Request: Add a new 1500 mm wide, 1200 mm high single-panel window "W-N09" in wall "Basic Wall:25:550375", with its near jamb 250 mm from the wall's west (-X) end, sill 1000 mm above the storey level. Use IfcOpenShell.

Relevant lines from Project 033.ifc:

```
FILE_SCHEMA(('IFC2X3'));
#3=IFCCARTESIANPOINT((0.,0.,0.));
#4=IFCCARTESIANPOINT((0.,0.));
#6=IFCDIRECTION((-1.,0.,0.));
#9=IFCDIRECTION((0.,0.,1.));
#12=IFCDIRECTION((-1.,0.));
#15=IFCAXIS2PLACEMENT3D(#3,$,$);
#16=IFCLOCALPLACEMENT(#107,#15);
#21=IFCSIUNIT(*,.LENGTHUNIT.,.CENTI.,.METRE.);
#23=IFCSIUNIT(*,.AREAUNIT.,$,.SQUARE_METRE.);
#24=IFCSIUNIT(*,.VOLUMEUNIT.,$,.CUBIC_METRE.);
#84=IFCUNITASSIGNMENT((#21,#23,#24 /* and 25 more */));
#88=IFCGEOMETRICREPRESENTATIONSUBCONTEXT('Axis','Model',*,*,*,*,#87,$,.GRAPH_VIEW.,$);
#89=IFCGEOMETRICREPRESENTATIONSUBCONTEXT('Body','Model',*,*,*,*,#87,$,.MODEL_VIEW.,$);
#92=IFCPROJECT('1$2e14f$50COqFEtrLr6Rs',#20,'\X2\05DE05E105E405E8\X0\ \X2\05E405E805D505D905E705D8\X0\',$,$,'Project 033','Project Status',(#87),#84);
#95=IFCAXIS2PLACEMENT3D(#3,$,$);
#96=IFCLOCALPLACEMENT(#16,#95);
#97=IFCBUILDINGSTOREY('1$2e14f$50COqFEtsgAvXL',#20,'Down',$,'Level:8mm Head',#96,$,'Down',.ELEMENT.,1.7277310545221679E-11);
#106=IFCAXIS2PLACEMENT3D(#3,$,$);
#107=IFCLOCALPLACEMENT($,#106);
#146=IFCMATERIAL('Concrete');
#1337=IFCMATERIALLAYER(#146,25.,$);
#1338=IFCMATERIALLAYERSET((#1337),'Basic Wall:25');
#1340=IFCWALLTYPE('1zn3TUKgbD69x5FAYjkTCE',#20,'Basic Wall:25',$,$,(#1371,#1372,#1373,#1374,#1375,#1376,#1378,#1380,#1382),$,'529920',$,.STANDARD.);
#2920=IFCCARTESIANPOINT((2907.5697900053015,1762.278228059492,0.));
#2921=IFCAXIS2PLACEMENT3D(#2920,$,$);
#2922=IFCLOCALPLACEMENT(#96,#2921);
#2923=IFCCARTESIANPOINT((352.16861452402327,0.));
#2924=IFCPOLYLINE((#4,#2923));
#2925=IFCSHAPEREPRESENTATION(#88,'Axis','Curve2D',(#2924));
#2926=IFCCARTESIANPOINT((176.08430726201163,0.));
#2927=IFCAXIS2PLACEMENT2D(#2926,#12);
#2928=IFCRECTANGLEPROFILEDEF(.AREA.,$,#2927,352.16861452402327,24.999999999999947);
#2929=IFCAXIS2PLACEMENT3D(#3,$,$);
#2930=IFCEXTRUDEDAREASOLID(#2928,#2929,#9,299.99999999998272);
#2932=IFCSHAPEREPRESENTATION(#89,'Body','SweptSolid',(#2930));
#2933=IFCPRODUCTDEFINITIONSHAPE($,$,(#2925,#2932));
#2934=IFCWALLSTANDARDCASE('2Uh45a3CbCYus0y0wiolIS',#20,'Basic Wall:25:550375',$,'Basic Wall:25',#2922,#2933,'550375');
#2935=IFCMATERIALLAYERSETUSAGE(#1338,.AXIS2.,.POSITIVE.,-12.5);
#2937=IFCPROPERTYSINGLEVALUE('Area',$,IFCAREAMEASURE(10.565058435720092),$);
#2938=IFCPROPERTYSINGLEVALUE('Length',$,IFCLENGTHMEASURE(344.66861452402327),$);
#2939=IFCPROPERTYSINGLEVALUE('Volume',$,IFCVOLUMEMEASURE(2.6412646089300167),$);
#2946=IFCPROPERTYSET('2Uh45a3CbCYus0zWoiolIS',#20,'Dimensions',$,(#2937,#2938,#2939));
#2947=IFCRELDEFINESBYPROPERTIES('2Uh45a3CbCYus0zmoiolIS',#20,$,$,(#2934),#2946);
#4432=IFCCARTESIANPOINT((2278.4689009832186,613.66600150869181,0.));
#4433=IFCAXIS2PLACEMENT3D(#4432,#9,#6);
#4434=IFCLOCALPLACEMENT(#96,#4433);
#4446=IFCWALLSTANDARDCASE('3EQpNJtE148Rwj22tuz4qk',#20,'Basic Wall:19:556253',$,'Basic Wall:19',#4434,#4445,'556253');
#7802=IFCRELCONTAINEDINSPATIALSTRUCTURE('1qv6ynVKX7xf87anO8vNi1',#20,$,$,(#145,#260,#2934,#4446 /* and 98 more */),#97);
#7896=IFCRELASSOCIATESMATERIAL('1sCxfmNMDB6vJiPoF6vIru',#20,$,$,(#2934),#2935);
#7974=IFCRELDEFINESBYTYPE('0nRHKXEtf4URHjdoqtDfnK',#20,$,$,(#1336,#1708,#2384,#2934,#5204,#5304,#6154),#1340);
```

```python
import numpy as np
import ifcopenshell
import ifcopenshell.api.feature
import ifcopenshell.api.geometry
import ifcopenshell.api.pset
import ifcopenshell.api.root
import ifcopenshell.api.spatial
import ifcopenshell.api.type
import ifcopenshell.geom
import ifcopenshell.util.element
import ifcopenshell.util.placement
import ifcopenshell.util.representation
import ifcopenshell.util.shape
import ifcopenshell.util.unit

model = ifcopenshell.open("Project 033.ifc")
unit_scale = ifcopenshell.util.unit.calculate_unit_scale(model)
area_scale = ifcopenshell.util.unit.calculate_unit_scale(model, "AREAUNIT")
volume_scale = ifcopenshell.util.unit.calculate_unit_scale(model, "VOLUMEUNIT")
settings = ifcopenshell.geom.settings()


def volume(element):
    """Net volume in cubic metres, openings subtracted."""
    shape = ifcopenshell.geom.create_shape(settings, element)
    return ifcopenshell.util.shape.get_volume(shape.geometry)


wall = model.by_guid("2Uh45a3CbCYus0y0wiolIS")
storey = ifcopenshell.util.element.get_container(wall, ifc_class="IfcBuildingStorey")
context = ifcopenshell.util.representation.get_context(model, "Model", "Body", "MODEL_VIEW")
before = volume(wall)

width, height, from_end, sill = 1.5, 1.2, 0.25, 1  # metres

# The wall runs along its own X axis, and the end named is its -X end.
wall_shape = ifcopenshell.geom.create_shape(settings, wall)
x, y, z = ifcopenshell.util.shape.get_vertices(wall_shape.geometry).T
start = x.min() + from_end
face, thickness = float(y.min()), float(y.max() - y.min())
wall_matrix = ifcopenshell.util.placement.get_local_placement(wall.ObjectPlacement)
level = ifcopenshell.util.placement.get_local_placement(storey.ObjectPlacement)[2, 3]


def in_wall(x, y):
    """Placement at x, y metres in the wall's axes, at sill height."""
    matrix = wall_matrix.copy()
    matrix[:, 3] = wall_matrix @ np.array([x / unit_scale, y / unit_scale, 0.0, 1.0])
    matrix[2, 3] = level + sill / unit_scale
    return matrix


# Opening: a box that overshoots both wall faces by 50 mm.
opening = ifcopenshell.api.root.create_entity(model, ifc_class="IfcOpeningElement")
box = ifcopenshell.api.geometry.add_wall_representation(
    model, context=context, length=width, height=height, thickness=thickness + 0.1
)
ifcopenshell.api.geometry.assign_representation(model, product=opening, representation=box)
ifcopenshell.api.geometry.edit_object_placement(model, product=opening, matrix=in_wall(start, face - 0.05), is_si=False)
ifcopenshell.api.feature.add_feature(model, feature=opening, element=wall)

window = ifcopenshell.api.root.create_entity(model, ifc_class="IfcWindow", name="W-N09")
window.OverallWidth, window.OverallHeight = width / unit_scale, height / unit_scale
body = ifcopenshell.api.geometry.add_window_representation(
    model,
    context=context,
    overall_width=window.OverallWidth,
    overall_height=window.OverallHeight,
    partition_type="SINGLE_PANEL",
)
ifcopenshell.api.geometry.assign_representation(model, product=window, representation=body)
ifcopenshell.api.spatial.assign_container(model, products=[window], relating_structure=storey)
fills = ifcopenshell.api.feature.add_filling(model, opening=opening, element=window)
fills.OwnerHistory = window.OwnerHistory  # required in IFC2X3

# IFC2X3 keeps the operation on the window style.
style = ifcopenshell.api.root.create_entity(model, ifc_class="IfcWindowStyle", name="W-N09")
style.OperationType, style.ConstructionType = "SINGLE_PANEL", "NOTDEFINED"
style.ParameterTakesPrecedence = style.Sizeable = False
ifcopenshell.api.type.assign_type(model, related_objects=[window], relating_type=style)

# Centre the window in the wall's thickness.
ifcopenshell.api.geometry.edit_object_placement(model, product=window, matrix=in_wall(start, face), is_si=False)
window_shape = ifcopenshell.geom.create_shape(settings, window)
depth = ifcopenshell.util.shape.get_vertices(window_shape.geometry)[:, 1]
offset = face + thickness / 2 - (depth.min() + depth.max()) / 2
ifcopenshell.api.geometry.edit_object_placement(model, product=window, matrix=in_wall(start, offset), is_si=False)

after = volume(wall)

# Update the wall's stored quantities.
pset = model.by_id(ifcopenshell.util.element.get_pset(wall, "Dimensions", should_inherit=False)["id"])
ifcopenshell.api.pset.edit_pset(model, pset=pset, properties={
    "Area": model.create_entity("IfcAreaMeasure", after / thickness / area_scale),
    "Volume": model.create_entity("IfcVolumeMeasure", after / volume_scale),
})

print(f"wall volume {before:.3f} -> {after:.3f} m3")

model.write("Project 033_updated.ifc")
```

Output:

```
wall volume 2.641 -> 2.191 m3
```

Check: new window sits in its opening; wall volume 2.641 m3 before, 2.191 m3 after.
